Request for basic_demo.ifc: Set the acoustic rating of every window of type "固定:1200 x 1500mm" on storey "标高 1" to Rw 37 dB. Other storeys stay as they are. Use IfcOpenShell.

First a look at what the model holds.

```python
import ifcopenshell
import ifcopenshell.util.element

model = ifcopenshell.open("basic_demo.ifc")
print(model.schema)
storey = next(s for s in model.by_type("IfcBuildingStorey") if s.Name == "标高 1")
windows = [e for e in ifcopenshell.util.element.get_decomposition(storey) if e.is_a("IfcWindow")]
seen = {}
for e in windows:
    element_type = ifcopenshell.util.element.get_type(e)
    key = (element_type.Name if element_type != e and element_type else None, ifcopenshell.util.element.get_pset(e, "Pset_WindowCommon", "AcousticRating"))
    seen[key] = seen.get(key, 0) + 1
for (name, value), count in sorted(seen.items(), key=str):
    print(count, "x", name, "|", value)
```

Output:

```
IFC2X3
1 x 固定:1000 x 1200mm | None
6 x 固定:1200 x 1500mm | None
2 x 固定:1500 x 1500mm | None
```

```python
import ifcopenshell
import ifcopenshell.api.pset
import ifcopenshell.util.element

model = ifcopenshell.open("basic_demo.ifc")

storey = next(s for s in model.by_type("IfcBuildingStorey") if s.Name == "标高 1")
windows = [e for e in ifcopenshell.util.element.get_decomposition(storey) if e.is_a("IfcWindow")]

count = 0
for e in windows:
    element_type = ifcopenshell.util.element.get_type(e)
    if element_type in (None, e) or element_type.Name != "固定:1200 x 1500mm":
        continue
    # add_pset returns the element's existing set when there is one.
    pset = ifcopenshell.api.pset.add_pset(model, product=e, name="Pset_WindowCommon")
    ifcopenshell.api.pset.edit_pset(model, pset=pset, properties={"AcousticRating": "Rw 37 dB"})
    count += 1

print(count, "windows updated")

model.write("basic_demo_edited.ifc")
```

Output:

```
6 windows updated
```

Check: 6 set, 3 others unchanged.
